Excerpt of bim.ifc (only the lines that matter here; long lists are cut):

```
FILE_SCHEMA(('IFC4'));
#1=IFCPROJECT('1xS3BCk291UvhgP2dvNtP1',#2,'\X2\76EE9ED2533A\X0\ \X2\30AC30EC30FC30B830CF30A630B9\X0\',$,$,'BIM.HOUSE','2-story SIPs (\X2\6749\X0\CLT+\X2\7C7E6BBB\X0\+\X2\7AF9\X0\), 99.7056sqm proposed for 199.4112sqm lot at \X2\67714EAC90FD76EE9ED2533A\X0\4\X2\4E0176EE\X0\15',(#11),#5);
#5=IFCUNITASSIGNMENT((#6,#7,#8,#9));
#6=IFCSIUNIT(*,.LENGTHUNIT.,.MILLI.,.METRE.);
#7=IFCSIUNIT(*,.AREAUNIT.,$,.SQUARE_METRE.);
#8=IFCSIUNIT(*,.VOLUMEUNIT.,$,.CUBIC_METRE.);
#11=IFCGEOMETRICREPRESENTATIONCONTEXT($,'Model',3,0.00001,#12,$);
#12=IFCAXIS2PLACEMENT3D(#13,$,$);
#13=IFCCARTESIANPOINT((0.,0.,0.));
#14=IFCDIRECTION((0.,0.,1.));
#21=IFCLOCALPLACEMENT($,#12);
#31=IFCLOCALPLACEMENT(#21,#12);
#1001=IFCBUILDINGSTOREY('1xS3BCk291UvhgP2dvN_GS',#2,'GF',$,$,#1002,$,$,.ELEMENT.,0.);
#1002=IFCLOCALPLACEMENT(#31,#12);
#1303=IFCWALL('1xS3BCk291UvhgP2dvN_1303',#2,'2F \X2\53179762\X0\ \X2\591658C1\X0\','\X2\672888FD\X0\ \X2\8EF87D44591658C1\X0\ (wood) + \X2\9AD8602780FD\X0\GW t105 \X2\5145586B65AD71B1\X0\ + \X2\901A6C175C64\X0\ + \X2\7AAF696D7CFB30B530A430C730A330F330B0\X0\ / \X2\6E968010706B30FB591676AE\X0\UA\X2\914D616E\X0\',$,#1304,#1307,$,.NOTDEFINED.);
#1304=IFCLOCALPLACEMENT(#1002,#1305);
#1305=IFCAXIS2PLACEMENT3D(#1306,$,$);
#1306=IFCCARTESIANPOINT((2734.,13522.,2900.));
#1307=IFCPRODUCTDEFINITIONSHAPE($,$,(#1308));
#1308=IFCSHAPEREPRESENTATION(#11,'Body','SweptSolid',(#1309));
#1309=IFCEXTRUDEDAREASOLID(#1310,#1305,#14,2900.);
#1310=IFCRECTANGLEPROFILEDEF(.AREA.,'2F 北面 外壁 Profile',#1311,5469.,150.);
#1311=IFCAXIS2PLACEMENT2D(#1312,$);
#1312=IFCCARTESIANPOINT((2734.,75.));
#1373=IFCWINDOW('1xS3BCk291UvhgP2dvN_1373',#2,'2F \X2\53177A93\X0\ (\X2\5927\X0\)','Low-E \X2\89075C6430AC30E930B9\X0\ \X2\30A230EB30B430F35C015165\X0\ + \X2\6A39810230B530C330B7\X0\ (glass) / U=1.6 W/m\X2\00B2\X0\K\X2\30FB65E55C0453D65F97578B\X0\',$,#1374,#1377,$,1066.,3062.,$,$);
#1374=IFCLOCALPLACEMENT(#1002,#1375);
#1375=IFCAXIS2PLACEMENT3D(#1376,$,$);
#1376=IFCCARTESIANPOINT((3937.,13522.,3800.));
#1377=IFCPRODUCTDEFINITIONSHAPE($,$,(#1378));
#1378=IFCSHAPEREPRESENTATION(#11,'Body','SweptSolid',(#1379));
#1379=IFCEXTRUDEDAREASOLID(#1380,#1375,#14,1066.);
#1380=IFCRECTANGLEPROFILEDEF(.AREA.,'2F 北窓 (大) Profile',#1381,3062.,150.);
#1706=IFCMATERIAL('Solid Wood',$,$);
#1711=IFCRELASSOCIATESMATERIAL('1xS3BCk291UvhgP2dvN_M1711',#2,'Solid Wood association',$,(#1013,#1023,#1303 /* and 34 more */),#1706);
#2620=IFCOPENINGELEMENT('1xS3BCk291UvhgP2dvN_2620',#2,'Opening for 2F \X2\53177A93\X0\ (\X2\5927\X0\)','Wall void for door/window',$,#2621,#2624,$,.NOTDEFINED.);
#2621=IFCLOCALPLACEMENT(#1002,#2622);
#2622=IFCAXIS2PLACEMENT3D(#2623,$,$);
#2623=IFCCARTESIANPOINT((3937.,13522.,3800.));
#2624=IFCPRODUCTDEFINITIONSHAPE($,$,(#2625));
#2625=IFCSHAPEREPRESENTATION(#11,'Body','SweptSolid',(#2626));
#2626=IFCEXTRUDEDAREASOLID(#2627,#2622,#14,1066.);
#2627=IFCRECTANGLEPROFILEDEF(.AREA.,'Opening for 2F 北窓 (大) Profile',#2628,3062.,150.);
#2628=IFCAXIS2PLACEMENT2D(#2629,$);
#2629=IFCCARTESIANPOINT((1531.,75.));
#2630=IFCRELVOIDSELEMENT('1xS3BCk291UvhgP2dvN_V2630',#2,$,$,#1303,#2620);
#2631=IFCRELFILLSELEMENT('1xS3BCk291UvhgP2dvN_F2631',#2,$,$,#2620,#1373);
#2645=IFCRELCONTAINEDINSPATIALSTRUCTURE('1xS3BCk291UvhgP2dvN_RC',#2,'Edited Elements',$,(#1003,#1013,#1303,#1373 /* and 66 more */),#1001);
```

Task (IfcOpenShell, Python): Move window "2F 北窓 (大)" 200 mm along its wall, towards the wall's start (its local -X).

```python
import ifcopenshell
import ifcopenshell.api.geometry
import ifcopenshell.util.placement
import ifcopenshell.util.unit

model = ifcopenshell.open("bim.ifc")
unit_scale = ifcopenshell.util.unit.calculate_unit_scale(model)

window = model.by_guid("1xS3BCk291UvhgP2dvN_1373")
opening = window.FillsVoids[0].RelatingOpeningElement
wall = opening.VoidsElements[0].RelatingBuildingElement

wall_matrix = ifcopenshell.util.placement.get_local_placement(wall.ObjectPlacement)
shift = wall_matrix[:3, 0] * -0.2 / unit_scale
before = ifcopenshell.util.placement.get_local_placement(window.ObjectPlacement)[:3, 3].copy()

# The window is not placed relative to its opening, so move both.
for product in (opening, window):
    matrix = ifcopenshell.util.placement.get_local_placement(product.ObjectPlacement)
    matrix[:3, 3] += shift
    ifcopenshell.api.geometry.edit_object_placement(model, product=product, matrix=matrix, is_si=False)

after = ifcopenshell.util.placement.get_local_placement(window.ObjectPlacement)[:3, 3]
print("window moved by", (after - before).round(3) + 0.0)

model.write("bim_v2.ifc")
```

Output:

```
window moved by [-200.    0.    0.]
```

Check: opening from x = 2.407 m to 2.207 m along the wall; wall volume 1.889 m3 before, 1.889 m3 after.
